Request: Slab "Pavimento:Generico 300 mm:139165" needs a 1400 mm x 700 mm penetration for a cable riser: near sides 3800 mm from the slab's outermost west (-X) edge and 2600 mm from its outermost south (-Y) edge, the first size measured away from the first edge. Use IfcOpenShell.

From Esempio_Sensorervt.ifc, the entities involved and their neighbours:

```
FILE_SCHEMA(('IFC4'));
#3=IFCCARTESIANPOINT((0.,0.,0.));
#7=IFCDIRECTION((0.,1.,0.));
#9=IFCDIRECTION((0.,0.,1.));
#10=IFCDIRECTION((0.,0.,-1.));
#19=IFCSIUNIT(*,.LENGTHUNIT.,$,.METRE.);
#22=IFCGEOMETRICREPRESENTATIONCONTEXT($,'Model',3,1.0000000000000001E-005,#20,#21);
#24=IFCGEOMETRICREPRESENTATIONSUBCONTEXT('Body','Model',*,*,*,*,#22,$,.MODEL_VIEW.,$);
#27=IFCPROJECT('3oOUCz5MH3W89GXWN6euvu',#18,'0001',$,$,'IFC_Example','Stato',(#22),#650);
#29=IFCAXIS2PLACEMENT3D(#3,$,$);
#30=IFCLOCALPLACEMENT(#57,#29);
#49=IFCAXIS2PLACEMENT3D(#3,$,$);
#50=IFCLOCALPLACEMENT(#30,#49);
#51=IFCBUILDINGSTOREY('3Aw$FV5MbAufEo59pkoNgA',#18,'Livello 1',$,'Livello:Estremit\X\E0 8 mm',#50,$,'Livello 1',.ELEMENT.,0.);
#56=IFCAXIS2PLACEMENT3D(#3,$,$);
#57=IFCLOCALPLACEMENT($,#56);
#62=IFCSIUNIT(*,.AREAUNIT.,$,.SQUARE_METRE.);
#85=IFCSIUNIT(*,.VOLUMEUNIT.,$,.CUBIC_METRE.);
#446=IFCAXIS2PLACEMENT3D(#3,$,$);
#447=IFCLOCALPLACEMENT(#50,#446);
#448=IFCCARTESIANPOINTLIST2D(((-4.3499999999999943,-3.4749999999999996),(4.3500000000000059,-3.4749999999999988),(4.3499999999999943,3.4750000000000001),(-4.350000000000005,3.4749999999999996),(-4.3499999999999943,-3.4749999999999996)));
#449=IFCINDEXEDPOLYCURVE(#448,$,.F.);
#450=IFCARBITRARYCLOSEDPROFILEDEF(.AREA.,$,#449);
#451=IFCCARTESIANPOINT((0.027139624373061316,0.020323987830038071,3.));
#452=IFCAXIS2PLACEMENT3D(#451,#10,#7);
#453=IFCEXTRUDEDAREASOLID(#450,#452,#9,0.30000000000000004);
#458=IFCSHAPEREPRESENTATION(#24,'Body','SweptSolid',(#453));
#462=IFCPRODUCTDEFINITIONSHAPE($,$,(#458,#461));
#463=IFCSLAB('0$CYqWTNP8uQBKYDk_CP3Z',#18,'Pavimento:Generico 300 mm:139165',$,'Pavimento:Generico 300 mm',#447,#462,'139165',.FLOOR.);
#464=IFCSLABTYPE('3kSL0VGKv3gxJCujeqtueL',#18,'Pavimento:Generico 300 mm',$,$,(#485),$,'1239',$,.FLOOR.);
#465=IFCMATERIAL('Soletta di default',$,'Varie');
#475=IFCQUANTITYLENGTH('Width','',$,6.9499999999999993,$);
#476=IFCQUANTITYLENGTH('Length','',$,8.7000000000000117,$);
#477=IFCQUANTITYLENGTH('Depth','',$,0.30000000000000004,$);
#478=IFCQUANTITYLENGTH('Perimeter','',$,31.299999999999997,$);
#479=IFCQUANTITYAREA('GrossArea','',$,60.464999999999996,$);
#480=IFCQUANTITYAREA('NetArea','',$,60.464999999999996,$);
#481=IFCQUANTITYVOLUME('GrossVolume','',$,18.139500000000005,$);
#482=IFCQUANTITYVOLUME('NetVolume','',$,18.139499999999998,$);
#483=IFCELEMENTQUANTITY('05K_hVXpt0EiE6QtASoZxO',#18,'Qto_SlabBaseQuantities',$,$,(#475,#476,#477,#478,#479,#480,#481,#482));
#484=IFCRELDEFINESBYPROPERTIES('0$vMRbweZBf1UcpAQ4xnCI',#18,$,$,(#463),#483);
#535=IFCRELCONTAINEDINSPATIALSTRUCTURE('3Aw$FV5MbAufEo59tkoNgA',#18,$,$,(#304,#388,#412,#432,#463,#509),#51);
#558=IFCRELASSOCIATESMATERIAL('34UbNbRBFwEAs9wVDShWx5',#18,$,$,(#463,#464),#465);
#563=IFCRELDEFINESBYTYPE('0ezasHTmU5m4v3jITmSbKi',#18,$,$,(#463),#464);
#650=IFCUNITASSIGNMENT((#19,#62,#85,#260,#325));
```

```python
import numpy as np
import ifcopenshell
import ifcopenshell.api.feature
import ifcopenshell.api.geometry
import ifcopenshell.api.pset
import ifcopenshell.api.root
import ifcopenshell.geom
import ifcopenshell.util.element
import ifcopenshell.util.placement
import ifcopenshell.util.representation
import ifcopenshell.util.shape
import ifcopenshell.util.unit

model = ifcopenshell.open("Esempio_Sensorervt.ifc")
unit_scale = ifcopenshell.util.unit.calculate_unit_scale(model)
area_scale = ifcopenshell.util.unit.calculate_unit_scale(model, "AREAUNIT")
volume_scale = ifcopenshell.util.unit.calculate_unit_scale(model, "VOLUMEUNIT")
settings = ifcopenshell.geom.settings()


def volume(element):
    """Net volume in cubic metres, openings subtracted."""
    shape = ifcopenshell.geom.create_shape(settings, element)
    return ifcopenshell.util.shape.get_volume(shape.geometry)


slab = model.by_id(463)
before = volume(slab)

# Extent in the slab's own axes, in metres. The edges named are its -X and -Y sides.
slab_shape = ifcopenshell.geom.create_shape(settings, slab)
vertices = ifcopenshell.util.shape.get_vertices(slab_shape.geometry)
x_min, y_min, bottom = vertices.min(axis=0)
top = vertices[:, 2].max()

opening = ifcopenshell.api.root.create_entity(model, ifc_class="IfcOpeningElement", name="Cable riser opening", predefined_type="OPENING")
context = ifcopenshell.util.representation.get_context(model, "Model", "Body", "MODEL_VIEW")
width, depth = 1.4, 0.7
outline = [(0.0, 0.0), (width, 0.0), (width, depth), (0.0, depth), (0.0, 0.0)]
# Overshoot both faces by 50 mm so the cut is clean.
shape = ifcopenshell.api.geometry.add_slab_representation(
    model, context=context, depth=top - bottom + 0.1, polyline=outline
)
ifcopenshell.api.geometry.assign_representation(model, product=opening, representation=shape)

matrix = ifcopenshell.util.placement.get_local_placement(slab.ObjectPlacement)
matrix[:, 3] = matrix @ np.append(np.array([x_min + 3.8, y_min + 2.6, bottom - 0.05]) / unit_scale, 1.0)
ifcopenshell.api.geometry.edit_object_placement(model, product=opening, matrix=matrix, is_si=False)
ifcopenshell.api.feature.add_feature(model, feature=opening, element=slab)

after = volume(slab)

# Update the slab's stored quantities.
qto = model.by_id(ifcopenshell.util.element.get_pset(slab, "Qto_SlabBaseQuantities", should_inherit=False)["id"])
ifcopenshell.api.pset.edit_qto(model, qto=qto, properties={
    "NetArea": after / (top - bottom) / area_scale,
    "NetVolume": after / volume_scale,
})

print(f"slab volume {before:.3f} -> {after:.3f} m3")

model.write("Esempio_Sensorervt_updated.ifc")
```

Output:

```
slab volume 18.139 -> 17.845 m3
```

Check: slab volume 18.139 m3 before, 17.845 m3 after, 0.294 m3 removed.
